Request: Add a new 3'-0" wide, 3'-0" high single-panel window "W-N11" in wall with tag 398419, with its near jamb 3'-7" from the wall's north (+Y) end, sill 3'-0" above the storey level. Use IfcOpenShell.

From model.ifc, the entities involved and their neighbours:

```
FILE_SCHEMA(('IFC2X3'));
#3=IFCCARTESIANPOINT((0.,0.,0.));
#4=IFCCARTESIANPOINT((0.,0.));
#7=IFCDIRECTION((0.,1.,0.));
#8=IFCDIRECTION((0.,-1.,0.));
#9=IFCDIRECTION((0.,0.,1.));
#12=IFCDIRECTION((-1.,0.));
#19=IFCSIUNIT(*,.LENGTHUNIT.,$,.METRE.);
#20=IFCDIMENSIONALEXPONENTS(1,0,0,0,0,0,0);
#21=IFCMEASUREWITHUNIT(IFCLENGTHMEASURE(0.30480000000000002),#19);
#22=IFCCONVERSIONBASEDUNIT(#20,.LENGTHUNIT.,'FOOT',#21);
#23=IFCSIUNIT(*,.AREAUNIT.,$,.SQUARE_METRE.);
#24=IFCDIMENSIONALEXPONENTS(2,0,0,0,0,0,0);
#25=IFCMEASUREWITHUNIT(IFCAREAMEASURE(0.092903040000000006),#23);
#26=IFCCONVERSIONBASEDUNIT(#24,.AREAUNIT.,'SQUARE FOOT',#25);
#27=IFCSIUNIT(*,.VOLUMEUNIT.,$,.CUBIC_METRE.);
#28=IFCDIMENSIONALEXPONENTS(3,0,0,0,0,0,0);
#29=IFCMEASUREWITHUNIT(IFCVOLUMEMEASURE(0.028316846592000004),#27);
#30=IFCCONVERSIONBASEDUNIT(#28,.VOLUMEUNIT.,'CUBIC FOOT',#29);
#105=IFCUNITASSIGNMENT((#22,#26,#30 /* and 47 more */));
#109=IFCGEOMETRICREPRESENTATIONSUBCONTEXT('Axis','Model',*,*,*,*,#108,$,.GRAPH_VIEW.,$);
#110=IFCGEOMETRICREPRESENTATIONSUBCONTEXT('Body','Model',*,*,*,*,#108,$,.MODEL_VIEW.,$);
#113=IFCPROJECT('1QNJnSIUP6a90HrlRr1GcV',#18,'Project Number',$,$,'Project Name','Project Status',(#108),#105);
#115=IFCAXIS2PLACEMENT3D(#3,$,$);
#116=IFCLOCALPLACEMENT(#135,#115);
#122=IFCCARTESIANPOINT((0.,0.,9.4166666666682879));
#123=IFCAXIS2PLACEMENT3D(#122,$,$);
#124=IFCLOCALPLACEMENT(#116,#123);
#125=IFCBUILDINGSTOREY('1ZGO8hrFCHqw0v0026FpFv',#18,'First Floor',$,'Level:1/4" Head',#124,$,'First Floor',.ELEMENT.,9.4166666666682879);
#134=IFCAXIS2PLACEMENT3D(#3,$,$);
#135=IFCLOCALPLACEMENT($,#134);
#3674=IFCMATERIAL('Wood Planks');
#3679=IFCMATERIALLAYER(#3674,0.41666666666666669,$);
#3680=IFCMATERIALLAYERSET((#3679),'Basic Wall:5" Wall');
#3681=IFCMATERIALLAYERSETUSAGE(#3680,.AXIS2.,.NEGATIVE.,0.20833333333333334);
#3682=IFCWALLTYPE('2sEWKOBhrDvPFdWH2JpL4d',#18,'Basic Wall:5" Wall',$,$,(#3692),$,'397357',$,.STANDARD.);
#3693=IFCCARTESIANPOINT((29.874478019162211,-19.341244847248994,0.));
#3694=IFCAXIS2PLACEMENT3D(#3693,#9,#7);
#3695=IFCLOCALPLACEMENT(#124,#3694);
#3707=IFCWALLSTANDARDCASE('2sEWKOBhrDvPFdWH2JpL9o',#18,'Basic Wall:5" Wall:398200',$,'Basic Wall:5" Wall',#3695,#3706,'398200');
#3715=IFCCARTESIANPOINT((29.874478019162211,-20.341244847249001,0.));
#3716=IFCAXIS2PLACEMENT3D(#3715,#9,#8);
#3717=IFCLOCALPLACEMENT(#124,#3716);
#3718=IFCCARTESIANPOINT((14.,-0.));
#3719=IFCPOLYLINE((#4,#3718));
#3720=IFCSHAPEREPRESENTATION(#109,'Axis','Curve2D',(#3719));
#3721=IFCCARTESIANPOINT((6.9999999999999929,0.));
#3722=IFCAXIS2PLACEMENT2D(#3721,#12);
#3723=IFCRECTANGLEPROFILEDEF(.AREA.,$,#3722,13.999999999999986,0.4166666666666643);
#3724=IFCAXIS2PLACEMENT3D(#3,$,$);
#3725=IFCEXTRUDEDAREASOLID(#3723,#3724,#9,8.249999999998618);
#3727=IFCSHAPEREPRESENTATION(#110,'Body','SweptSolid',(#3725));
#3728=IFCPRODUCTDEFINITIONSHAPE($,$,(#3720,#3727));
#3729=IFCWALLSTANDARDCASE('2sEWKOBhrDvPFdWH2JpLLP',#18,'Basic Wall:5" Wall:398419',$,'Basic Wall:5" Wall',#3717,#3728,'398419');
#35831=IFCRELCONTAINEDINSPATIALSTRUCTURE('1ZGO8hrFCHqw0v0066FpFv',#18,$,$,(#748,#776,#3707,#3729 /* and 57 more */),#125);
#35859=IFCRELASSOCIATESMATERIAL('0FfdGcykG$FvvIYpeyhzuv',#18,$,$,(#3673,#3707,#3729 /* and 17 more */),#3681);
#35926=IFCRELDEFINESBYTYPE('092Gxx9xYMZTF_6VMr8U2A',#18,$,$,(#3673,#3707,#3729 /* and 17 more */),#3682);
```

```python
import numpy as np
import ifcopenshell
import ifcopenshell.api.feature
import ifcopenshell.api.geometry
import ifcopenshell.api.root
import ifcopenshell.api.spatial
import ifcopenshell.api.type
import ifcopenshell.geom
import ifcopenshell.util.element
import ifcopenshell.util.placement
import ifcopenshell.util.representation
import ifcopenshell.util.shape
import ifcopenshell.util.unit

model = ifcopenshell.open("model.ifc")
unit_scale = ifcopenshell.util.unit.calculate_unit_scale(model)
settings = ifcopenshell.geom.settings()


def volume(element):
    """Net volume in cubic metres, openings subtracted."""
    shape = ifcopenshell.geom.create_shape(settings, element)
    return ifcopenshell.util.shape.get_volume(shape.geometry)


wall = model.by_guid("2sEWKOBhrDvPFdWH2JpLLP")
storey = ifcopenshell.util.element.get_container(wall, ifc_class="IfcBuildingStorey")
context = ifcopenshell.util.representation.get_context(model, "Model", "Body", "MODEL_VIEW")
before = volume(wall)

width, height, from_end, sill = 0.9144, 0.9144, 1.0922, 0.9144  # metres

# The wall runs along its own X axis, and the end named is its -X end.
wall_shape = ifcopenshell.geom.create_shape(settings, wall)
x, y, z = ifcopenshell.util.shape.get_vertices(wall_shape.geometry).T
start = x.min() + from_end
face, thickness = float(y.min()), float(y.max() - y.min())
wall_matrix = ifcopenshell.util.placement.get_local_placement(wall.ObjectPlacement)
level = ifcopenshell.util.placement.get_local_placement(storey.ObjectPlacement)[2, 3]


def in_wall(x, y):
    """Placement at x, y metres in the wall's axes, at sill height."""
    matrix = wall_matrix.copy()
    matrix[:, 3] = wall_matrix @ np.array([x / unit_scale, y / unit_scale, 0.0, 1.0])
    matrix[2, 3] = level + sill / unit_scale
    return matrix


# Opening: a box that overshoots both wall faces by 50 mm.
opening = ifcopenshell.api.root.create_entity(model, ifc_class="IfcOpeningElement")
box = ifcopenshell.api.geometry.add_wall_representation(
    model, context=context, length=width, height=height, thickness=thickness + 0.1
)
ifcopenshell.api.geometry.assign_representation(model, product=opening, representation=box)
ifcopenshell.api.geometry.edit_object_placement(model, product=opening, matrix=in_wall(start, face - 0.05), is_si=False)
ifcopenshell.api.feature.add_feature(model, feature=opening, element=wall)

window = ifcopenshell.api.root.create_entity(model, ifc_class="IfcWindow", name="W-N11")
window.OverallWidth, window.OverallHeight = width / unit_scale, height / unit_scale
body = ifcopenshell.api.geometry.add_window_representation(
    model,
    context=context,
    overall_width=window.OverallWidth,
    overall_height=window.OverallHeight,
    partition_type="SINGLE_PANEL",
)
ifcopenshell.api.geometry.assign_representation(model, product=window, representation=body)
ifcopenshell.api.spatial.assign_container(model, products=[window], relating_structure=storey)
fills = ifcopenshell.api.feature.add_filling(model, opening=opening, element=window)
fills.OwnerHistory = window.OwnerHistory  # required in IFC2X3

# IFC2X3 keeps the operation on the window style.
style = ifcopenshell.api.root.create_entity(model, ifc_class="IfcWindowStyle", name="W-N11")
style.OperationType, style.ConstructionType = "SINGLE_PANEL", "NOTDEFINED"
style.ParameterTakesPrecedence = style.Sizeable = False
ifcopenshell.api.type.assign_type(model, related_objects=[window], relating_type=style)

# Centre the window in the wall's thickness.
ifcopenshell.api.geometry.edit_object_placement(model, product=window, matrix=in_wall(start, face), is_si=False)
window_shape = ifcopenshell.geom.create_shape(settings, window)
depth = ifcopenshell.util.shape.get_vertices(window_shape.geometry)[:, 1]
offset = face + thickness / 2 - (depth.min() + depth.max()) / 2
ifcopenshell.api.geometry.edit_object_placement(model, product=window, matrix=in_wall(start, offset), is_si=False)

after = volume(wall)

print(f"wall volume {before:.3f} -> {after:.3f} m3")

model.write("model_updated.ifc")
```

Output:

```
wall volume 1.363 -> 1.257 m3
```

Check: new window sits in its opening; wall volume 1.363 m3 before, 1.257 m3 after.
